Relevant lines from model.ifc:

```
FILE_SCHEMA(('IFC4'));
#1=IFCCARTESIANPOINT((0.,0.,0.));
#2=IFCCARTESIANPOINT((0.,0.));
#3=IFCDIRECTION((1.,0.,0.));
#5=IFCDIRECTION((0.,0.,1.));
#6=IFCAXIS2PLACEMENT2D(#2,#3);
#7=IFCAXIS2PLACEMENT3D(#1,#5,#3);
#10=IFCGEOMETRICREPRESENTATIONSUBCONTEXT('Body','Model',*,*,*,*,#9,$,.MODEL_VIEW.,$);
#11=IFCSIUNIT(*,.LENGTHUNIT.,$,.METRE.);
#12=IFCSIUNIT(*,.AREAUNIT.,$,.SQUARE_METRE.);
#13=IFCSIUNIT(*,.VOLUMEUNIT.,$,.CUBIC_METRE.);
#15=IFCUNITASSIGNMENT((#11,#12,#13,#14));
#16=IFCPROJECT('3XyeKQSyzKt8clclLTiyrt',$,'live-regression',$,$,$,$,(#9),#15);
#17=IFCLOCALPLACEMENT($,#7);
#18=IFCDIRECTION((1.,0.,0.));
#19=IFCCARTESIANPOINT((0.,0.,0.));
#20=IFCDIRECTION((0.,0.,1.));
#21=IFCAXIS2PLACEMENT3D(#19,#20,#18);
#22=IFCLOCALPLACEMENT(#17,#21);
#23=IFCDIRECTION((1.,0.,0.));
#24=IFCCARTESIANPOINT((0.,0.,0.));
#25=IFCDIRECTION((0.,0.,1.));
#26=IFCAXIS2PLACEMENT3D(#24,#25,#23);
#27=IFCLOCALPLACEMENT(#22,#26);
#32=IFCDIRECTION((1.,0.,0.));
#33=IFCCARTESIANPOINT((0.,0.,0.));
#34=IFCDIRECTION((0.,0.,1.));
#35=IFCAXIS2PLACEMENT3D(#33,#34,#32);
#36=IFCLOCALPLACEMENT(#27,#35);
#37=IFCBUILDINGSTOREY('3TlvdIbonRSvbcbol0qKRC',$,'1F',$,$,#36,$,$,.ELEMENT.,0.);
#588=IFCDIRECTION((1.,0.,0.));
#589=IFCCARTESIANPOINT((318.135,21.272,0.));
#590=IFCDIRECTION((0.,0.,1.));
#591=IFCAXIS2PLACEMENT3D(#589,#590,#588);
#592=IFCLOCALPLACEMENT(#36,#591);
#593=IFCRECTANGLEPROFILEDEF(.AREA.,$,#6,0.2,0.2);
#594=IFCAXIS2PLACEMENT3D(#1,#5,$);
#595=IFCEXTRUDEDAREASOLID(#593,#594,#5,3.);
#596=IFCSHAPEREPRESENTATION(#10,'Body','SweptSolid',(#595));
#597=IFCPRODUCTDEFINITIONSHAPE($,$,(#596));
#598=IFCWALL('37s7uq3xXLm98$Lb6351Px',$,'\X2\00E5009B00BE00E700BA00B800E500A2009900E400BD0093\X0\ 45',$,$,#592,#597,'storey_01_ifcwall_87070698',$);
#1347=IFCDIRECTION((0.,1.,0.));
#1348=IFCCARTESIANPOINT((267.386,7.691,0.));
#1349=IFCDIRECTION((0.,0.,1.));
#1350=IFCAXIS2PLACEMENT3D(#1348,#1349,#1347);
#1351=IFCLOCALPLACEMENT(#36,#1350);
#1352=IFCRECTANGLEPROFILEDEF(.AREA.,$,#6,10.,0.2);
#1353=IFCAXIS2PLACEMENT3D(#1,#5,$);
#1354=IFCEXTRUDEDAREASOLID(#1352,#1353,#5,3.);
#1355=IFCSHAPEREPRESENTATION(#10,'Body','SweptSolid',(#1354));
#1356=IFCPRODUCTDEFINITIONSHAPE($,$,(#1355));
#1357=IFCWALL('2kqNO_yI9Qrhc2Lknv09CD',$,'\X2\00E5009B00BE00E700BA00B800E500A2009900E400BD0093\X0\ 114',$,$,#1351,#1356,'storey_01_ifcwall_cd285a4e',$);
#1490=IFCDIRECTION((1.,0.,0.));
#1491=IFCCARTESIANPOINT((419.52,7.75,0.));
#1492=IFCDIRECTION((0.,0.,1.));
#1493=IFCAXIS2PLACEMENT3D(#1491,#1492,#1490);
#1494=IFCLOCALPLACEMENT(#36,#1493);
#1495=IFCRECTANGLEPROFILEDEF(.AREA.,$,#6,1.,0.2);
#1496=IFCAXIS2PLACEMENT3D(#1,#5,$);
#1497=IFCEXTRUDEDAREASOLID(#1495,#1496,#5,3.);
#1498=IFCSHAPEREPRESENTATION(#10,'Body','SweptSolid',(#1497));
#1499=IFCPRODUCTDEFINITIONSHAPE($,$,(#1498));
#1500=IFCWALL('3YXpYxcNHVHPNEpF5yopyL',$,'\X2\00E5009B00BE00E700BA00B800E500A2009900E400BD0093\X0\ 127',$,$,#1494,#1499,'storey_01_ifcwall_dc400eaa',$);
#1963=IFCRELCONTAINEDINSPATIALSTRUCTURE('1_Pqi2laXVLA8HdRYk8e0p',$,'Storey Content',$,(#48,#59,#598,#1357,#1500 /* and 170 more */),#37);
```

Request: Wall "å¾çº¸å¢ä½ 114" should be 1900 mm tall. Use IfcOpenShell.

```python
import ifcopenshell
import ifcopenshell.geom
import ifcopenshell.util.representation
import ifcopenshell.util.shape

model = ifcopenshell.open("model.ifc")
settings = ifcopenshell.geom.settings()


def volume(element):
    """Net volume in cubic metres, openings subtracted."""
    shape = ifcopenshell.geom.create_shape(settings, element)
    return ifcopenshell.util.shape.get_volume(shape.geometry)


wall = model.by_id(1357)
before = volume(wall)

body = ifcopenshell.util.representation.get_representation(wall, "Model", "Body")
solid = body.Items[0]
old_height = solid.Depth
solid.Depth = 1.9
after = volume(wall)

print(f"height {old_height:g} -> {solid.Depth:g}, volume {before:.3f} -> {after:.3f} m3")

model.write("model-out.ifc")
```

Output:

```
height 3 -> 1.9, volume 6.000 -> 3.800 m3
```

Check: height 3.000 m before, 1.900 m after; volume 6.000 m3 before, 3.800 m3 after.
